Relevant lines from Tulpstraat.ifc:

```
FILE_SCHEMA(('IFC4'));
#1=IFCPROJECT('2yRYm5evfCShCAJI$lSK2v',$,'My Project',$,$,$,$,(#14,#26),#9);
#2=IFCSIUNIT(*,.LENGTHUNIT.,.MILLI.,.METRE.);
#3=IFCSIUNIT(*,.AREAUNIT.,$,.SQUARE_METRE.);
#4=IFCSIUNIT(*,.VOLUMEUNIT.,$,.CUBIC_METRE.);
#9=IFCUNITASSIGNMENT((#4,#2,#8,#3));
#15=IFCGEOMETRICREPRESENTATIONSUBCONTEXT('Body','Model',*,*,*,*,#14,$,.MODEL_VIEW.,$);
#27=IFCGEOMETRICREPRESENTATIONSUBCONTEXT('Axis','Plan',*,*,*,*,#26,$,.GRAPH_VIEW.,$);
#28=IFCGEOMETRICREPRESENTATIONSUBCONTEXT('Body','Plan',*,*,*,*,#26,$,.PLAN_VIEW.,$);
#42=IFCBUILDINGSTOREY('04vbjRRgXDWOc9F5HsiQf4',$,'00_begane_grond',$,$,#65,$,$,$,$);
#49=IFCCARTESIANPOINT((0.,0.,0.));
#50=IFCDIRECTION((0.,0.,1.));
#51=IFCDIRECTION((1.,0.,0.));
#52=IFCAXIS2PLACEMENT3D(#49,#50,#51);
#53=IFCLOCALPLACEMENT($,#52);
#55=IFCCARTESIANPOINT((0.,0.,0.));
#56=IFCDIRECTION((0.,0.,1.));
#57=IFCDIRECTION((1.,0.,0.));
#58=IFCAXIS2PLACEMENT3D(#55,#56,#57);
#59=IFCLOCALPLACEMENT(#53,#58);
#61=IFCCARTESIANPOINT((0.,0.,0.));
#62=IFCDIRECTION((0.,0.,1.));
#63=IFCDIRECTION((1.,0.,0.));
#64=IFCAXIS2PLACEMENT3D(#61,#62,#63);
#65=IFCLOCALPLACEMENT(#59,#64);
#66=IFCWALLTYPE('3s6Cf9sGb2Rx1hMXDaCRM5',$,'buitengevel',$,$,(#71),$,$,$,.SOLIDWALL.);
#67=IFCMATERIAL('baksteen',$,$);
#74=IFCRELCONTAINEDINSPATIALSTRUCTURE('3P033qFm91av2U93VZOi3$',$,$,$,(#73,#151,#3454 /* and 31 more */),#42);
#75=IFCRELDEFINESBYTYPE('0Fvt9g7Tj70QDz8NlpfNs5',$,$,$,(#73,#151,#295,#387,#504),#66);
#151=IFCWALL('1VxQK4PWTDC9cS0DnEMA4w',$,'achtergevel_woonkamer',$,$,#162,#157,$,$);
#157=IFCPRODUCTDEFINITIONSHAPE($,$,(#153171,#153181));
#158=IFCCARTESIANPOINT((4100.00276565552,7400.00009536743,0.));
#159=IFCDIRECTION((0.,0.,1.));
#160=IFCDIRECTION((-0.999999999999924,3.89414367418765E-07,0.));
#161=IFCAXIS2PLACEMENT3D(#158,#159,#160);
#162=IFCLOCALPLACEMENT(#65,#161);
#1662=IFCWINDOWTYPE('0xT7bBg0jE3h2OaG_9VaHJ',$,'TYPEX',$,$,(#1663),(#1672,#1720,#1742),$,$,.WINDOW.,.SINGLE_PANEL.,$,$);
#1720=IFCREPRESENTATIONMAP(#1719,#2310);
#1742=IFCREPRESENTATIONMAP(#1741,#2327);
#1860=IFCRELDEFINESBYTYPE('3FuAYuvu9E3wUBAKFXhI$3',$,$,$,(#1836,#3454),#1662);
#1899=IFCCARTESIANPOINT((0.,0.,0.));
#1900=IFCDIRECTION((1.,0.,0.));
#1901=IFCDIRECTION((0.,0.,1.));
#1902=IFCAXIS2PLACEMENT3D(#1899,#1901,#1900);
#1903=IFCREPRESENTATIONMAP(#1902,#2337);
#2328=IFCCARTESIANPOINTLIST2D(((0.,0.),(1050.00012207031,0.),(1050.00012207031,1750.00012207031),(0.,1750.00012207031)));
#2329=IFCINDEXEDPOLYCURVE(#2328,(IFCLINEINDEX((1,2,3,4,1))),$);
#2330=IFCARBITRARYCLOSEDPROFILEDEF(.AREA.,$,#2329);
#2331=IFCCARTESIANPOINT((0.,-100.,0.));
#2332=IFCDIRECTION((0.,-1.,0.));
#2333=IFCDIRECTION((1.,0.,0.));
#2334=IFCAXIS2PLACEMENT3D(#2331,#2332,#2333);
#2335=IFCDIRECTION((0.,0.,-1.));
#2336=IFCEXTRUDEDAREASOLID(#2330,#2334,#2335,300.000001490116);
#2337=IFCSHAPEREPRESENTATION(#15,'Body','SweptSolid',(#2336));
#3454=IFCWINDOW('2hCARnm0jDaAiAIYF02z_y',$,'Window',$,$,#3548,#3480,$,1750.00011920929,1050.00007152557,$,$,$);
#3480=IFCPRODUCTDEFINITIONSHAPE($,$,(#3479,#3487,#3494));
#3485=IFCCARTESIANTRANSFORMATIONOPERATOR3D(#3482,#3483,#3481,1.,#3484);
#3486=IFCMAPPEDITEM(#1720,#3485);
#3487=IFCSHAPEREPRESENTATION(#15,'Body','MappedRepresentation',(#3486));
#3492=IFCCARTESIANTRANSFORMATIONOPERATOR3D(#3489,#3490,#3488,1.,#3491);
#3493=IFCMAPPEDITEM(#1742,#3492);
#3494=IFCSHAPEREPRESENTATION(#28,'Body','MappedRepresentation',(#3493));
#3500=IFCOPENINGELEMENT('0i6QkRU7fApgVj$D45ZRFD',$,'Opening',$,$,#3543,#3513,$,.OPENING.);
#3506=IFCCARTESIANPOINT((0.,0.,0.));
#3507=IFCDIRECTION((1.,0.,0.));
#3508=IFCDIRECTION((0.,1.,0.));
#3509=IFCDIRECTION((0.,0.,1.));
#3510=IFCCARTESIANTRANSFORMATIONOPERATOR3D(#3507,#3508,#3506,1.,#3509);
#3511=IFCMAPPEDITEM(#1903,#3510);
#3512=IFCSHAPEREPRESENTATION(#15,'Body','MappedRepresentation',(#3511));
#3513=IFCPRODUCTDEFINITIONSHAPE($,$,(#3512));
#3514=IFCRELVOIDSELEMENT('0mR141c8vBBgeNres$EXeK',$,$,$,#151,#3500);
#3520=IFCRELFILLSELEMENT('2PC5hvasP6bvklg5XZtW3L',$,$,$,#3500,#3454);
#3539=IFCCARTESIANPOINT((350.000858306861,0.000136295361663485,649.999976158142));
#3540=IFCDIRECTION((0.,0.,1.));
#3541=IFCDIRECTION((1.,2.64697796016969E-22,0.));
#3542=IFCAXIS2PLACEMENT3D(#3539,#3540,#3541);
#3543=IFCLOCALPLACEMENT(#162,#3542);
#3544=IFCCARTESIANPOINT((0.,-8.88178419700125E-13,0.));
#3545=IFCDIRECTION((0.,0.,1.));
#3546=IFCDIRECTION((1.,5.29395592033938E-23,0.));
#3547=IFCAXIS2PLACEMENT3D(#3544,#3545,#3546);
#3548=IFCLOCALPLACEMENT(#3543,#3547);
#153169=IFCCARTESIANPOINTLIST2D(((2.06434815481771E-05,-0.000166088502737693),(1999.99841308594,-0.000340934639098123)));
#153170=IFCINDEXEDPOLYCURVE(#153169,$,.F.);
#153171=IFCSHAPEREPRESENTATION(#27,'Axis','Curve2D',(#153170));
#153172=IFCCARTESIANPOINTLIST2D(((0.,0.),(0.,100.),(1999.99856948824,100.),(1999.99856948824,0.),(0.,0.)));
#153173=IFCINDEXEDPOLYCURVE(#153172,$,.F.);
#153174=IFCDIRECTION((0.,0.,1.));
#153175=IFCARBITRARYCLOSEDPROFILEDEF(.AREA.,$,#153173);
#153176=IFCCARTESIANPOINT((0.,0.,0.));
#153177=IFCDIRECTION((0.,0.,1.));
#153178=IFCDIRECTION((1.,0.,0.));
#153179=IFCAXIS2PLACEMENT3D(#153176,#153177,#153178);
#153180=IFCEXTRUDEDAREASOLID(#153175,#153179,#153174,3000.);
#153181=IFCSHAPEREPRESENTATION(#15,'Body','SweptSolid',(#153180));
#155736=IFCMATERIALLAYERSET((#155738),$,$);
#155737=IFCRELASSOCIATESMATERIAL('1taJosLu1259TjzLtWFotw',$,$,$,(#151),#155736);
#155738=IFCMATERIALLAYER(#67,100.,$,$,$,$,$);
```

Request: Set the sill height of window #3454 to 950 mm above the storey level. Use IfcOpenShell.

```python
import numpy as np
import ifcopenshell
import ifcopenshell.api.geometry
import ifcopenshell.geom
import ifcopenshell.util.element
import ifcopenshell.util.placement
import ifcopenshell.util.shape
import ifcopenshell.util.unit

model = ifcopenshell.open("Tulpstraat.ifc")
unit_scale = ifcopenshell.util.unit.calculate_unit_scale(model)

window = model.by_id(3454)
opening = window.FillsVoids[0].RelatingOpeningElement
storey = ifcopenshell.util.element.get_container(window, ifc_class="IfcBuildingStorey")
level = ifcopenshell.util.placement.get_local_placement(storey.ObjectPlacement)[2, 3]

# The opening's origin need not be at the sill, so measure its lowest point.
shape = ifcopenshell.geom.create_shape(ifcopenshell.geom.settings(), opening)
bottom = ifcopenshell.util.shape.get_shape_bottom_elevation(shape, shape.geometry) / unit_scale
dz = level + 0.95 / unit_scale - bottom

shift = np.array([0.0, 0.0, dz])
# The window is placed relative to its opening, so it follows when the opening moves.
matrix = ifcopenshell.util.placement.get_local_placement(opening.ObjectPlacement)
matrix[:3, 3] += shift
ifcopenshell.api.geometry.edit_object_placement(
    model, product=opening, matrix=matrix, is_si=False, should_transform_children=True
)

print(f"moved by {dz * unit_scale:+.3f} m")

model.write("Tulpstraat_updated.ifc")
```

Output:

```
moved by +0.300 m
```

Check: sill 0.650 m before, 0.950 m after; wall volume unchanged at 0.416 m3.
